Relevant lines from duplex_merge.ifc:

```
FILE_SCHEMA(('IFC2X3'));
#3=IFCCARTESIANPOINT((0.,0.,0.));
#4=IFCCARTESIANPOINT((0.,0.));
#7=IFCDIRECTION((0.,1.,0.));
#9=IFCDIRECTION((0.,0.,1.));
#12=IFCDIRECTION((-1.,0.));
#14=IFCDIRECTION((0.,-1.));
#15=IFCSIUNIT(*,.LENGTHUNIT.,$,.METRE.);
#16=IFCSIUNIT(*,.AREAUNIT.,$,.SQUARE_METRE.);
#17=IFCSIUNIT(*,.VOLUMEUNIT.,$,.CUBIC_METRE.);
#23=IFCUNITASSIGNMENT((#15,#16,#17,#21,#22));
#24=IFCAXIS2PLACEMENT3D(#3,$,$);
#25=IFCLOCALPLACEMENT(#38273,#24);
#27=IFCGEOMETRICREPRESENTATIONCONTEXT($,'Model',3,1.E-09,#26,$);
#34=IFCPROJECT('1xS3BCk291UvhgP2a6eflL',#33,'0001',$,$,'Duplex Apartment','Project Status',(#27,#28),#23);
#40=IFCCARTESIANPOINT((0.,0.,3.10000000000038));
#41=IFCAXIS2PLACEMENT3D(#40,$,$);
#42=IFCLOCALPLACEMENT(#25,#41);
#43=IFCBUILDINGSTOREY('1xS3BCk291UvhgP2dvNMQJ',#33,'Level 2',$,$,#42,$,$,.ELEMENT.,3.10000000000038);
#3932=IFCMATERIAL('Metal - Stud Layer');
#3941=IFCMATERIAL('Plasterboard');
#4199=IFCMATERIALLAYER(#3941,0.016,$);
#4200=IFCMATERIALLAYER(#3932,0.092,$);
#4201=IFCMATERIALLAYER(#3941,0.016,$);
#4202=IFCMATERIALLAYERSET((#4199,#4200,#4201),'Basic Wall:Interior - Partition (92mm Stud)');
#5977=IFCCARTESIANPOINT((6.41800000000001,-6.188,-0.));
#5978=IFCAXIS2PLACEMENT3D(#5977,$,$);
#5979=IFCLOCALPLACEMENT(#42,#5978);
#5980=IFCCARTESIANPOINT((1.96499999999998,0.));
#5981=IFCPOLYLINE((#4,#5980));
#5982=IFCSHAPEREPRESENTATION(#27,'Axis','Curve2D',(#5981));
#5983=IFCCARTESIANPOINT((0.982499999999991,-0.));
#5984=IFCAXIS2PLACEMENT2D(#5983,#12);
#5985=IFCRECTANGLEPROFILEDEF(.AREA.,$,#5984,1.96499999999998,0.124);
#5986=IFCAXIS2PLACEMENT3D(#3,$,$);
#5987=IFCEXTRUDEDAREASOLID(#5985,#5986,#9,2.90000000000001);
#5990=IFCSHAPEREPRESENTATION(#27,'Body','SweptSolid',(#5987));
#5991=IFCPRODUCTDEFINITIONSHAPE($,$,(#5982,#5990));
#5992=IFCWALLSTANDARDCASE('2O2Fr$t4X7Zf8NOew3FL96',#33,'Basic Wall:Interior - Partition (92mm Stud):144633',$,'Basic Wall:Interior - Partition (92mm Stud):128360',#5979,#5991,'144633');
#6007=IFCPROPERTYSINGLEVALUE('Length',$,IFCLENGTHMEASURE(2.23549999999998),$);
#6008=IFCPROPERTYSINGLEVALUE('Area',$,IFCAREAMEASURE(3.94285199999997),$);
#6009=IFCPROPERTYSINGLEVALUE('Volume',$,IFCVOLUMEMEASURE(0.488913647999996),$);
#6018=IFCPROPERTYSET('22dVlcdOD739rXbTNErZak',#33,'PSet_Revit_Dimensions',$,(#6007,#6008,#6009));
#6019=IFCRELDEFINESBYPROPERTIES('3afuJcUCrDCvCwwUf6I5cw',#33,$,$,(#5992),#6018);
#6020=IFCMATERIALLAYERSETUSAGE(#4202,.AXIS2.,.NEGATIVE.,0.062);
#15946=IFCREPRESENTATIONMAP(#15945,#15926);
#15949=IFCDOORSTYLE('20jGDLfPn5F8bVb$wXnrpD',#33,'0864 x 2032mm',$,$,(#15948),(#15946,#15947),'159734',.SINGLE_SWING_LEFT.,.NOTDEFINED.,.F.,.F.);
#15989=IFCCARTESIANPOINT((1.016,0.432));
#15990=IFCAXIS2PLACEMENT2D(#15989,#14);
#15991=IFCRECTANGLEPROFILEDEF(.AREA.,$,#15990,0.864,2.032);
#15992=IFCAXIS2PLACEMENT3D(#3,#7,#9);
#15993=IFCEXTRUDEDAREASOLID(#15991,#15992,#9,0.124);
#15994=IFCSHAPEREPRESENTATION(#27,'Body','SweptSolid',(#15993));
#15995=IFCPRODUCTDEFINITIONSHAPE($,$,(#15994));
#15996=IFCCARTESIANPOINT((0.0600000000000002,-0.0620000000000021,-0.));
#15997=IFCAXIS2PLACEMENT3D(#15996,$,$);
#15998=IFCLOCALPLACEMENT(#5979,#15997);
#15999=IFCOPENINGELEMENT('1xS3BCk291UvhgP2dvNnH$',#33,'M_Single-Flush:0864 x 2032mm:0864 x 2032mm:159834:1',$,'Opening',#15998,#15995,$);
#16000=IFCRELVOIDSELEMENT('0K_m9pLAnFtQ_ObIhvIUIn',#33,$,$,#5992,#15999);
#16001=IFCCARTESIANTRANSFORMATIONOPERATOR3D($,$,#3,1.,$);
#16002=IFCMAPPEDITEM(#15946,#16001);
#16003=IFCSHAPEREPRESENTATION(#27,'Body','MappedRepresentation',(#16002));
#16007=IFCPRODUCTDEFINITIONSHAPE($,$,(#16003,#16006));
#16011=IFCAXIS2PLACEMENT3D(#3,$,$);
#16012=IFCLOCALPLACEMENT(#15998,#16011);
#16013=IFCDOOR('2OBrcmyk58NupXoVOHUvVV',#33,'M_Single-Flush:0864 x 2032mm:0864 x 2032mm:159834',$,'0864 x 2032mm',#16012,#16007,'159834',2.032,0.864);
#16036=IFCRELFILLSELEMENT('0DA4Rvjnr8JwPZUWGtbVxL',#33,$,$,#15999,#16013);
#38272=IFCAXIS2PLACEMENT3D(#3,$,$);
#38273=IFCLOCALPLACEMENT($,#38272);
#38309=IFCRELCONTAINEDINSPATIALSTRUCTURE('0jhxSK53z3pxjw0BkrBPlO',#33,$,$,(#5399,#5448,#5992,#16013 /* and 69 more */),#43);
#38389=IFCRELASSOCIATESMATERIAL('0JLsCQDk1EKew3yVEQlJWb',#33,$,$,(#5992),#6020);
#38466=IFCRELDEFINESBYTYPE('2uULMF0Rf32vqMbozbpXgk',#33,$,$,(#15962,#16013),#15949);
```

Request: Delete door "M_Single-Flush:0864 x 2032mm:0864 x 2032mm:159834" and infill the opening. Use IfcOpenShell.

```python
import ifcopenshell
import ifcopenshell.api.feature
import ifcopenshell.api.pset
import ifcopenshell.api.root
import ifcopenshell.geom
import ifcopenshell.util.element
import ifcopenshell.util.shape
import ifcopenshell.util.unit

model = ifcopenshell.open("duplex_merge.ifc")
area_scale = ifcopenshell.util.unit.calculate_unit_scale(model, "AREAUNIT")
volume_scale = ifcopenshell.util.unit.calculate_unit_scale(model, "VOLUMEUNIT")
settings = ifcopenshell.geom.settings()


def volume(element):
    """Net volume in cubic metres, openings subtracted."""
    shape = ifcopenshell.geom.create_shape(settings, element)
    return ifcopenshell.util.shape.get_volume(shape.geometry)


door = model.by_guid("2OBrcmyk58NupXoVOHUvVV")
opening = door.FillsVoids[0].RelatingOpeningElement
wall = opening.VoidsElements[0].RelatingBuildingElement
before = volume(wall)

ifcopenshell.api.root.remove_product(model, product=door)
ifcopenshell.api.feature.remove_feature(model, feature=opening)

after = volume(wall)
thickness = 0.124  # wall thickness in metres

# Update the wall's stored quantities.
pset = model.by_id(ifcopenshell.util.element.get_pset(wall, "PSet_Revit_Dimensions", should_inherit=False)["id"])
ifcopenshell.api.pset.edit_pset(model, pset=pset, properties={
    "Area": model.create_entity("IfcAreaMeasure", after / thickness / area_scale),
    "Volume": model.create_entity("IfcVolumeMeasure", after / volume_scale),
})

print(f"wall volume {before:.3f} -> {after:.3f} m3")

model.write("duplex_merge_rev.ifc")
```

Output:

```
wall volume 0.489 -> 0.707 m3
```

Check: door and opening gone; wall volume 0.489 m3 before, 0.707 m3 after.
